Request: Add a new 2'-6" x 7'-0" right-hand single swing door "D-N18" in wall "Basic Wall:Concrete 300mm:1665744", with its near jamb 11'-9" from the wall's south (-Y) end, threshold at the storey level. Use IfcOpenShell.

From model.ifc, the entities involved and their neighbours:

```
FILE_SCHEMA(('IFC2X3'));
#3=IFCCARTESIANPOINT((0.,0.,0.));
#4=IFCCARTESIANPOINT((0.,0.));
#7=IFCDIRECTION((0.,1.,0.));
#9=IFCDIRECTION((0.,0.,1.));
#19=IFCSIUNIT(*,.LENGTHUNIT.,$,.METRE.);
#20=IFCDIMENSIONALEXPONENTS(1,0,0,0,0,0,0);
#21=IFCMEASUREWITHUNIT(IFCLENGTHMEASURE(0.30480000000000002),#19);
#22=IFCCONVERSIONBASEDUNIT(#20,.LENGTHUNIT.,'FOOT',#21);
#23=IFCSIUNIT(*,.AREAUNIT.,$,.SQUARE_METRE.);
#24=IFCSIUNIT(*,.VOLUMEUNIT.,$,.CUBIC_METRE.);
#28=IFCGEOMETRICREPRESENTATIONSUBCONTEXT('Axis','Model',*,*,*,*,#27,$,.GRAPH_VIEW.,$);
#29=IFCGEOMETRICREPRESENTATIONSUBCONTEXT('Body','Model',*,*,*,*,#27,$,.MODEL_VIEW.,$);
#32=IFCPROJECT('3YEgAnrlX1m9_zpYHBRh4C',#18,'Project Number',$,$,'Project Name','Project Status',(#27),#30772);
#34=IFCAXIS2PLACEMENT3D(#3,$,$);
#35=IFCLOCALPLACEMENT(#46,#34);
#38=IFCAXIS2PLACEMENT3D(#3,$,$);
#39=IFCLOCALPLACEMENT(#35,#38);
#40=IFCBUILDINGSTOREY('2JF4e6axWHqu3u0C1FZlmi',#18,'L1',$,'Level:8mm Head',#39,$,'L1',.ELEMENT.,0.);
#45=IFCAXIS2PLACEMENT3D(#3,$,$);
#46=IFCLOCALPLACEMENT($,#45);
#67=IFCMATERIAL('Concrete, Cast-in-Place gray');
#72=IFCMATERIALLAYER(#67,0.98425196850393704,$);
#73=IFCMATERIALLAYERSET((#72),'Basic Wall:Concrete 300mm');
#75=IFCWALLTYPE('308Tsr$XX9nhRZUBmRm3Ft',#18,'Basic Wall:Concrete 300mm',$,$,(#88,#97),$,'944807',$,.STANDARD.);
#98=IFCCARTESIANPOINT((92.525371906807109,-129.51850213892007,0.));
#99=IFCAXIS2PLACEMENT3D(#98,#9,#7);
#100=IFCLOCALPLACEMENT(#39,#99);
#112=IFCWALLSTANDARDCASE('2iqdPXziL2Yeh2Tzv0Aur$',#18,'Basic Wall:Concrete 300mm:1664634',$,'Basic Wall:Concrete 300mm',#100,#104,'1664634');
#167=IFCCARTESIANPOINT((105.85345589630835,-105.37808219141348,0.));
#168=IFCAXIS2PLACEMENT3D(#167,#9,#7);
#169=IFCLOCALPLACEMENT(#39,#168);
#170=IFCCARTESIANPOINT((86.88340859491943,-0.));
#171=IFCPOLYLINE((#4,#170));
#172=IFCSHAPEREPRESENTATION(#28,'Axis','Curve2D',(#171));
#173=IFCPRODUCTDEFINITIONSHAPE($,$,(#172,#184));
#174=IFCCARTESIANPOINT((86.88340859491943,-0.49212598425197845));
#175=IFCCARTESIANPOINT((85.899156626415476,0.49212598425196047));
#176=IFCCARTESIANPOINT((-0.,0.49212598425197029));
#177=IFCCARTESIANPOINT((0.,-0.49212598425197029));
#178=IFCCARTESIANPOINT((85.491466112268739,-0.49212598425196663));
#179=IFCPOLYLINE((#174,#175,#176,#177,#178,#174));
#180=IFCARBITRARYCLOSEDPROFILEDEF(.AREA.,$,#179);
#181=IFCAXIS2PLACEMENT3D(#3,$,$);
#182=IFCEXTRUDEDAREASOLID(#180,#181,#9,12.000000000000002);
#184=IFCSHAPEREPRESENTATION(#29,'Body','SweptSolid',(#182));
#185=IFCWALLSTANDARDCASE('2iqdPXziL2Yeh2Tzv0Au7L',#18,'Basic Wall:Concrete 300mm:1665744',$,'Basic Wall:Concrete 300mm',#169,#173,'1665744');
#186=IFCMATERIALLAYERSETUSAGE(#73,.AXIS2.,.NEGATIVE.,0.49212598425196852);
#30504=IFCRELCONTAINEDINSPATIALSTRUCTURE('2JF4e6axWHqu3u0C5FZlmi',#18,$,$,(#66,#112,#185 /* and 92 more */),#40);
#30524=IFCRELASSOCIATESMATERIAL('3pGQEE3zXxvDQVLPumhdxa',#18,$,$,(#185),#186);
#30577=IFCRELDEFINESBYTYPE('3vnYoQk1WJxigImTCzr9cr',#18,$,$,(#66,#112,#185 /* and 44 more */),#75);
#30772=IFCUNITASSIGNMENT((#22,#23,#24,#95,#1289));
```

```python
import numpy as np
import ifcopenshell
import ifcopenshell.api.feature
import ifcopenshell.api.geometry
import ifcopenshell.api.root
import ifcopenshell.api.spatial
import ifcopenshell.api.type
import ifcopenshell.geom
import ifcopenshell.util.element
import ifcopenshell.util.placement
import ifcopenshell.util.representation
import ifcopenshell.util.shape
import ifcopenshell.util.unit

model = ifcopenshell.open("model.ifc")
unit_scale = ifcopenshell.util.unit.calculate_unit_scale(model)
settings = ifcopenshell.geom.settings()


def volume(element):
    """Net volume in cubic metres, openings subtracted."""
    shape = ifcopenshell.geom.create_shape(settings, element)
    return ifcopenshell.util.shape.get_volume(shape.geometry)


wall = model.by_guid("2iqdPXziL2Yeh2Tzv0Au7L")
storey = ifcopenshell.util.element.get_container(wall, ifc_class="IfcBuildingStorey")
context = ifcopenshell.util.representation.get_context(model, "Model", "Body", "MODEL_VIEW")
before = volume(wall)

width, height, from_end, sill = 0.762, 2.1336, 3.5814, 0.0  # metres

# The wall runs along its own X axis, and the end named is its -X end.
wall_shape = ifcopenshell.geom.create_shape(settings, wall)
x, y, z = ifcopenshell.util.shape.get_vertices(wall_shape.geometry).T
start = x.min() + from_end
face, thickness = float(y.min()), float(y.max() - y.min())
wall_matrix = ifcopenshell.util.placement.get_local_placement(wall.ObjectPlacement)
level = ifcopenshell.util.placement.get_local_placement(storey.ObjectPlacement)[2, 3]


def in_wall(x, y):
    """Placement at x, y metres in the wall's axes, at sill height."""
    matrix = wall_matrix.copy()
    matrix[:, 3] = wall_matrix @ np.array([x / unit_scale, y / unit_scale, 0.0, 1.0])
    matrix[2, 3] = level + sill / unit_scale
    return matrix


# Opening: a box that overshoots both wall faces by 50 mm.
opening = ifcopenshell.api.root.create_entity(model, ifc_class="IfcOpeningElement")
box = ifcopenshell.api.geometry.add_wall_representation(
    model, context=context, length=width, height=height, thickness=thickness + 0.1
)
ifcopenshell.api.geometry.assign_representation(model, product=opening, representation=box)
ifcopenshell.api.geometry.edit_object_placement(model, product=opening, matrix=in_wall(start, face - 0.05), is_si=False)
ifcopenshell.api.feature.add_feature(model, feature=opening, element=wall)

door = ifcopenshell.api.root.create_entity(model, ifc_class="IfcDoor", name="D-N18")
door.OverallWidth, door.OverallHeight = width / unit_scale, height / unit_scale
body = ifcopenshell.api.geometry.add_door_representation(
    model,
    context=context,
    overall_width=door.OverallWidth,
    overall_height=door.OverallHeight,
    operation_type="SINGLE_SWING_RIGHT",
    lining_properties={"LiningDepth": thickness / unit_scale, "ThresholdDepth": thickness / unit_scale},
)
ifcopenshell.api.geometry.assign_representation(model, product=door, representation=body)
ifcopenshell.api.spatial.assign_container(model, products=[door], relating_structure=storey)
fills = ifcopenshell.api.feature.add_filling(model, opening=opening, element=door)
fills.OwnerHistory = door.OwnerHistory  # required in IFC2X3

# IFC2X3 keeps the operation on the door style.
style = ifcopenshell.api.root.create_entity(model, ifc_class="IfcDoorStyle", name="D-N18")
style.OperationType, style.ConstructionType = "SINGLE_SWING_RIGHT", "NOTDEFINED"
style.ParameterTakesPrecedence = style.Sizeable = False
ifcopenshell.api.type.assign_type(model, related_objects=[door], relating_type=style)

# The lining spans the wall, so the door starts at the wall face.
ifcopenshell.api.geometry.edit_object_placement(model, product=door, matrix=in_wall(start, face), is_si=False)

after = volume(wall)

print(f"wall volume {before:.3f} -> {after:.3f} m3")

model.write("model_v2.ifc")
```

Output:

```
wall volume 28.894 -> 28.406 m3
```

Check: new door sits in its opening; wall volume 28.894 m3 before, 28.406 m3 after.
